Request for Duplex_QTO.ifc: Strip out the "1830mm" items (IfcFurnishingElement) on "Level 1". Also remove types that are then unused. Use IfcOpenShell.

First a look at what the model holds.

```python
import ifcopenshell
import ifcopenshell.util.element

model = ifcopenshell.open("Duplex_QTO.ifc")
print(model.schema)
storey = next(s for s in model.by_type("IfcBuildingStorey") if s.Name == "Level 1")
furniture = [e for e in ifcopenshell.util.element.get_decomposition(storey) if e.is_a("IfcFurnishingElement")]
seen = {}
for e in furniture:
    element_type = ifcopenshell.util.element.get_type(e)
    name = element_type.Name if element_type not in (None, e) else None
    seen[name] = seen.get(name, 0) + 1
for name, count in sorted(seen.items(), key=str):
    print(count, "x", name)
```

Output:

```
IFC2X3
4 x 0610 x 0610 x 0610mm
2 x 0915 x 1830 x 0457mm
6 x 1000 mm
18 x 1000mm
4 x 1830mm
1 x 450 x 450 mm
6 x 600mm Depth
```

```python
import ifcopenshell
import ifcopenshell.api.root
import ifcopenshell.util.element

model = ifcopenshell.open("Duplex_QTO.ifc")

storey = next(s for s in model.by_type("IfcBuildingStorey") if s.Name == "Level 1")
furniture = [e for e in ifcopenshell.util.element.get_decomposition(storey) if e.is_a("IfcFurnishingElement")]
targets = [e for e in furniture if (t := ifcopenshell.util.element.get_type(e)) not in (None, e) and t.Name == "1830mm"]
types = {ifcopenshell.util.element.get_type(e) for e in targets} - {None, *targets}

for e in targets:
    ifcopenshell.api.root.remove_product(model, product=e)
print(len(targets), "removed")

unused = [t for t in types if not ifcopenshell.util.element.get_types(t)]
for t in unused:
    ifcopenshell.api.root.remove_product(model, product=t)
print(len(unused), "unused types removed")

model.write("Duplex_QTO_updated.ifc")
```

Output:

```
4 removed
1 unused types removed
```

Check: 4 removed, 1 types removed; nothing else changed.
